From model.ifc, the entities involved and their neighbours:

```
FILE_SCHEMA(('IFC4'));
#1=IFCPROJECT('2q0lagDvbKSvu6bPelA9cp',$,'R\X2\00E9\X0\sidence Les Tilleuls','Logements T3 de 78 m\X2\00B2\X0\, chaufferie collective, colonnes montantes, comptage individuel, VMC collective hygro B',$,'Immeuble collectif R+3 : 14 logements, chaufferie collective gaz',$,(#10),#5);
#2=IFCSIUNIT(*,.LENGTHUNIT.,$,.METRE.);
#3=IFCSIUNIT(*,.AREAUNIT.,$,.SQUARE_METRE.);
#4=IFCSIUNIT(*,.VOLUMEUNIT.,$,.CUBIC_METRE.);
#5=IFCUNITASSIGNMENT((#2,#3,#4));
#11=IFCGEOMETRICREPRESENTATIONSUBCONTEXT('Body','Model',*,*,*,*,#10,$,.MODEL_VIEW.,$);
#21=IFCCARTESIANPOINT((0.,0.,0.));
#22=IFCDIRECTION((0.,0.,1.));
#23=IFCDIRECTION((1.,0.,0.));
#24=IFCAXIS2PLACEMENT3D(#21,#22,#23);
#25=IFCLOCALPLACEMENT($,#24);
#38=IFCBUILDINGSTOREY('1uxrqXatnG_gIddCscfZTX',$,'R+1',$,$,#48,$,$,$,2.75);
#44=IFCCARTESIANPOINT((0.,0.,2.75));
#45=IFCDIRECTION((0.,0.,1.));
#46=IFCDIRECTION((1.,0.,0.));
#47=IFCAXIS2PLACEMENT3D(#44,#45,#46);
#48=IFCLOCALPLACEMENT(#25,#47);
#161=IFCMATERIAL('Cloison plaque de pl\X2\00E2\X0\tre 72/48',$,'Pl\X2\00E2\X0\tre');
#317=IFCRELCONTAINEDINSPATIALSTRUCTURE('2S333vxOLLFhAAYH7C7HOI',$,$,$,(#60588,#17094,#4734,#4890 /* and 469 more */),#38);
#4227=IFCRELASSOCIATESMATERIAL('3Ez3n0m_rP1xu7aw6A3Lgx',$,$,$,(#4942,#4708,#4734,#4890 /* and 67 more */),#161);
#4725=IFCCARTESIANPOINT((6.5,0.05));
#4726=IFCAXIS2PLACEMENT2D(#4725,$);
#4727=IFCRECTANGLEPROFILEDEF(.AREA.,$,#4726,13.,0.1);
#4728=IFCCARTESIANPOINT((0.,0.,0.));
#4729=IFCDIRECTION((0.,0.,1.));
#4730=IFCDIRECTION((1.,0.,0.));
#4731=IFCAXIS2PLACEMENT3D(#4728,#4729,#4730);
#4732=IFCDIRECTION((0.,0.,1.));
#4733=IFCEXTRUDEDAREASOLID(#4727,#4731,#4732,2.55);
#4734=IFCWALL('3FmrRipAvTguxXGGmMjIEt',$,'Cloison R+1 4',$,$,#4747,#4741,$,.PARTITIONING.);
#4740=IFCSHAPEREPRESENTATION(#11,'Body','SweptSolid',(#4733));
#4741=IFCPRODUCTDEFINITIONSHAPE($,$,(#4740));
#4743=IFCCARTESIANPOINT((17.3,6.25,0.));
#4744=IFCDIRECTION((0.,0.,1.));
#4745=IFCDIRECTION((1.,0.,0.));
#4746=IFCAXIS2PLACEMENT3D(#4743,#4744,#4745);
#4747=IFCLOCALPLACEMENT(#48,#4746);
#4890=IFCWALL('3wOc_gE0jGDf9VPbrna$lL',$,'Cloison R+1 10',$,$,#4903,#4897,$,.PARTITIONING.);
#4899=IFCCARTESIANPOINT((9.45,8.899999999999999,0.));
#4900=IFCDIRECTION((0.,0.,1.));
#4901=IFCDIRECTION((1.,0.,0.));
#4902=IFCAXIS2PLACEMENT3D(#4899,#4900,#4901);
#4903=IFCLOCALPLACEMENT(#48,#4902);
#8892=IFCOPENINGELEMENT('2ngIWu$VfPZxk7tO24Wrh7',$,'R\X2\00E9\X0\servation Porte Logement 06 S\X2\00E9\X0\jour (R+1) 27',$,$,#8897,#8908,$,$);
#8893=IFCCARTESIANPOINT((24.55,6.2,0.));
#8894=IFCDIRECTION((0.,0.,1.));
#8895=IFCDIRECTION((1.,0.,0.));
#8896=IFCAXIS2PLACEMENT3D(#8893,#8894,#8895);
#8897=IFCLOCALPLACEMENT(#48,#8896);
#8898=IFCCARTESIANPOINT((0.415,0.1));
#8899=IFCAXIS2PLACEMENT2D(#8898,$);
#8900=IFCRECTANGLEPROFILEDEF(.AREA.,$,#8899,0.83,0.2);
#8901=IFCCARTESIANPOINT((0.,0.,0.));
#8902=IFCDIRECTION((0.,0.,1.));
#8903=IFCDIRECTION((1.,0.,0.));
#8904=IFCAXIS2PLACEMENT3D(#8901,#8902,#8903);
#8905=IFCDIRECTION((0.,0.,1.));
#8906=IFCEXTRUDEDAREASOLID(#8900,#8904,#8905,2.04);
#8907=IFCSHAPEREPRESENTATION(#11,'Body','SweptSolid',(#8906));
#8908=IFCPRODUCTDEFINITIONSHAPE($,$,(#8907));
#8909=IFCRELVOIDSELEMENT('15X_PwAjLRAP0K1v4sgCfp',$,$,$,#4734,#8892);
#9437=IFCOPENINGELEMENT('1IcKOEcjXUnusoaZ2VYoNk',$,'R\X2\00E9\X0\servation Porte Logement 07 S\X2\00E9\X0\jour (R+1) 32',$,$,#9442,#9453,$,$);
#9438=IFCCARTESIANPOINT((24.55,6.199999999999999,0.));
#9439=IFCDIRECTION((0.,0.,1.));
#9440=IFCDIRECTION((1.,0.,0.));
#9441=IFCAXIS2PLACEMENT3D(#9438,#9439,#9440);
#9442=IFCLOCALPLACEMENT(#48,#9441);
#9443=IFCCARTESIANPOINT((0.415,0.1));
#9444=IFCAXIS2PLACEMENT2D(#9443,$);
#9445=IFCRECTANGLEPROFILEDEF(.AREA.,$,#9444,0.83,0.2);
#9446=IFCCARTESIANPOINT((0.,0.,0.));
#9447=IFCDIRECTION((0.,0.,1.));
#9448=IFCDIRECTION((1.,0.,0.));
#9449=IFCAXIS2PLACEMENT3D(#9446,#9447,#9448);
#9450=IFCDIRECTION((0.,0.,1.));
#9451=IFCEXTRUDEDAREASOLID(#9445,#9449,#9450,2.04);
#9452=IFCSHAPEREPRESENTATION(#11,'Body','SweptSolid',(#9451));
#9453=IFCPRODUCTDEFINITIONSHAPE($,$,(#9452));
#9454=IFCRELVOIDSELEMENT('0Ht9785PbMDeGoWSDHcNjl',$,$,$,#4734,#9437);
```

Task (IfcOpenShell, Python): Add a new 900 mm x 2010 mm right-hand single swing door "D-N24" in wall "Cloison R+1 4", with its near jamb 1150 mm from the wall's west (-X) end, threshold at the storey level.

```python
import numpy as np
import ifcopenshell
import ifcopenshell.api.feature
import ifcopenshell.api.geometry
import ifcopenshell.api.root
import ifcopenshell.api.spatial
import ifcopenshell.geom
import ifcopenshell.util.element
import ifcopenshell.util.placement
import ifcopenshell.util.representation
import ifcopenshell.util.shape
import ifcopenshell.util.unit

model = ifcopenshell.open("model.ifc")
unit_scale = ifcopenshell.util.unit.calculate_unit_scale(model)
settings = ifcopenshell.geom.settings()


def volume(element):
    """Net volume in cubic metres, openings subtracted."""
    shape = ifcopenshell.geom.create_shape(settings, element)
    return ifcopenshell.util.shape.get_volume(shape.geometry)


wall = model.by_guid("3FmrRipAvTguxXGGmMjIEt")
storey = ifcopenshell.util.element.get_container(wall, ifc_class="IfcBuildingStorey")
context = ifcopenshell.util.representation.get_context(model, "Model", "Body", "MODEL_VIEW")
before = volume(wall)

width, height, from_end, sill = 0.9, 2.01, 1.15, 0.0  # metres

# The wall runs along its own X axis, and the end named is its -X end.
wall_shape = ifcopenshell.geom.create_shape(settings, wall)
x, y, z = ifcopenshell.util.shape.get_vertices(wall_shape.geometry).T
start = x.min() + from_end
face, thickness = float(y.min()), float(y.max() - y.min())
wall_matrix = ifcopenshell.util.placement.get_local_placement(wall.ObjectPlacement)
level = ifcopenshell.util.placement.get_local_placement(storey.ObjectPlacement)[2, 3]


def in_wall(x, y):
    """Placement at x, y metres in the wall's axes, at sill height."""
    matrix = wall_matrix.copy()
    matrix[:, 3] = wall_matrix @ np.array([x / unit_scale, y / unit_scale, 0.0, 1.0])
    matrix[2, 3] = level + sill / unit_scale
    return matrix


# Opening: a box that overshoots both wall faces by 50 mm.
opening = ifcopenshell.api.root.create_entity(model, ifc_class="IfcOpeningElement", predefined_type="OPENING")
box = ifcopenshell.api.geometry.add_wall_representation(
    model, context=context, length=width, height=height, thickness=thickness + 0.1
)
ifcopenshell.api.geometry.assign_representation(model, product=opening, representation=box)
ifcopenshell.api.geometry.edit_object_placement(model, product=opening, matrix=in_wall(start, face - 0.05), is_si=False)
ifcopenshell.api.feature.add_feature(model, feature=opening, element=wall)

door = ifcopenshell.api.root.create_entity(model, ifc_class="IfcDoor", name="D-N24", predefined_type="DOOR")
door.OverallWidth, door.OverallHeight = width / unit_scale, height / unit_scale
door.OperationType = "SINGLE_SWING_RIGHT"
body = ifcopenshell.api.geometry.add_door_representation(
    model,
    context=context,
    overall_width=door.OverallWidth,
    overall_height=door.OverallHeight,
    operation_type="SINGLE_SWING_RIGHT",
    lining_properties={"LiningDepth": thickness / unit_scale, "ThresholdDepth": thickness / unit_scale},
)
ifcopenshell.api.geometry.assign_representation(model, product=door, representation=body)
ifcopenshell.api.spatial.assign_container(model, products=[door], relating_structure=storey)
ifcopenshell.api.feature.add_filling(model, opening=opening, element=door)

# The lining spans the wall, so the door starts at the wall face.
ifcopenshell.api.geometry.edit_object_placement(model, product=door, matrix=in_wall(start, face), is_si=False)

after = volume(wall)

print(f"wall volume {before:.3f} -> {after:.3f} m3")

model.write("model_v2.ifc")
```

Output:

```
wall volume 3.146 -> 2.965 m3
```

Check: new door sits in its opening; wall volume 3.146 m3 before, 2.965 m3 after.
